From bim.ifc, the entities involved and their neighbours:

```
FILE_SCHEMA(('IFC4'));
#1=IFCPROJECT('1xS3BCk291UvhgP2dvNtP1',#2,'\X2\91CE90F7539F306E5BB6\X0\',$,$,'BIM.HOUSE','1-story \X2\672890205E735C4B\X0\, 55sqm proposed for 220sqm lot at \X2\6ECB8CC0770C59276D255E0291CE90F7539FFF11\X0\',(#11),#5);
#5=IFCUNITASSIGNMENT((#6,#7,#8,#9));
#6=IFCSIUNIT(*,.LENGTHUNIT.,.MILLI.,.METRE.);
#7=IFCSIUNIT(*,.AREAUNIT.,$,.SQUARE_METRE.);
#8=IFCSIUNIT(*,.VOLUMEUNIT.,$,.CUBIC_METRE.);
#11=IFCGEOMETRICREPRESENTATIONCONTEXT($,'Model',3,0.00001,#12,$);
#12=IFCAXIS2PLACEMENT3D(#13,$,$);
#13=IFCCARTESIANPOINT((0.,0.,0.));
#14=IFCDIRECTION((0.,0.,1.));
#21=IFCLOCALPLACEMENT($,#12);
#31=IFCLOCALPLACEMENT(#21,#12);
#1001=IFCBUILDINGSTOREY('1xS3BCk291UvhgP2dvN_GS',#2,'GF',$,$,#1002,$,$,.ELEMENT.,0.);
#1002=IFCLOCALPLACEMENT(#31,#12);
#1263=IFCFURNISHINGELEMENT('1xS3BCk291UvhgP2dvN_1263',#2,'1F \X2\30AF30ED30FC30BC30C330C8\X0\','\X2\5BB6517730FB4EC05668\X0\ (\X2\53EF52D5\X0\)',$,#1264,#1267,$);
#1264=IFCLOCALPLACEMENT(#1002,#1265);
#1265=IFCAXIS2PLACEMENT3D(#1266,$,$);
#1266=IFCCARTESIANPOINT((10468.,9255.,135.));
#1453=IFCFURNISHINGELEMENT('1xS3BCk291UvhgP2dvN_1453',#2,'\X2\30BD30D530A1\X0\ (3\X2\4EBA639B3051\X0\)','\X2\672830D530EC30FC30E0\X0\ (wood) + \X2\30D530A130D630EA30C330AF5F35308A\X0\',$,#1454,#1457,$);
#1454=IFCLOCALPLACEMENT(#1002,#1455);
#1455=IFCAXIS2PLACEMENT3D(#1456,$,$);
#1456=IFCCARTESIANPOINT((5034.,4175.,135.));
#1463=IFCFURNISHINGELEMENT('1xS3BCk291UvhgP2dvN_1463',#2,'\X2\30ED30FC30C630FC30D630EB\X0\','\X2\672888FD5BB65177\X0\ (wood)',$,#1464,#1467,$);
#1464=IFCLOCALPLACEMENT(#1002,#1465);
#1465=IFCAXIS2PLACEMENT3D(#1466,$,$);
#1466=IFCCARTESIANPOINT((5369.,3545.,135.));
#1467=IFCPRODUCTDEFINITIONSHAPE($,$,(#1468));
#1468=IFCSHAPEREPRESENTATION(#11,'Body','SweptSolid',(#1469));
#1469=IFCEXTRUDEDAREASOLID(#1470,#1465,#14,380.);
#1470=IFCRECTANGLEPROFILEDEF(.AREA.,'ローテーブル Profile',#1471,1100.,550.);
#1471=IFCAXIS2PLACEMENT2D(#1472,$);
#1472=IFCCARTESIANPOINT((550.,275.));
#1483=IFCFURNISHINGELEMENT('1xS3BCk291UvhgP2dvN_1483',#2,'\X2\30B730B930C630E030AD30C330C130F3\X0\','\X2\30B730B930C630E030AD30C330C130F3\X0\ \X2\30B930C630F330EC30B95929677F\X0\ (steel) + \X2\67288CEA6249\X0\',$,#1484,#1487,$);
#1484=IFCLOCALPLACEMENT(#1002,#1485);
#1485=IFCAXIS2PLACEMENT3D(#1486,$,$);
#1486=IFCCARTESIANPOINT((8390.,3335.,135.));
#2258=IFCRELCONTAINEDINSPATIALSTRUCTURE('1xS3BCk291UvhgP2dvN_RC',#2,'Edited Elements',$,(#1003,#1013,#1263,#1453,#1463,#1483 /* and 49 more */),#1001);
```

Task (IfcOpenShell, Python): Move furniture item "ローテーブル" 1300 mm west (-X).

```python
import ifcopenshell
import ifcopenshell.api.geometry
import ifcopenshell.util.placement

model = ifcopenshell.open("bim.ifc")

item = model.by_guid("1xS3BCk291UvhgP2dvN_1463")
matrix = ifcopenshell.util.placement.get_local_placement(item.ObjectPlacement)
matrix[0, 3] -= 1300.0
ifcopenshell.api.geometry.edit_object_placement(model, product=item, matrix=matrix, is_si=False)

print(ifcopenshell.util.placement.get_local_placement(item.ObjectPlacement).round(3) + 0.0)

model.write("bim_updated.ifc")
```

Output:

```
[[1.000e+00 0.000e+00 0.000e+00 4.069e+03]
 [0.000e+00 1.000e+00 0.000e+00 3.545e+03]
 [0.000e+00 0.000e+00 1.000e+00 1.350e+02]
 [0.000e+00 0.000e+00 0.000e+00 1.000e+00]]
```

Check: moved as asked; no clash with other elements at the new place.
